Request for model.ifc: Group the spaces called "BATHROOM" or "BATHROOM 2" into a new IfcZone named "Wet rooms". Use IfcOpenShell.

First a look at what the model holds.

```python
import ifcopenshell

model = ifcopenshell.open("model.ifc")
print(model.schema)
seen = {}
for space in model.by_type("IfcSpace"):
    seen[space.LongName] = seen.get(space.LongName, 0) + 1
for name, count in sorted(seen.items(), key=str):
    print(count, "x", name)
print("zones:", [z.Name for z in model.by_type("IfcZone")][:20])
```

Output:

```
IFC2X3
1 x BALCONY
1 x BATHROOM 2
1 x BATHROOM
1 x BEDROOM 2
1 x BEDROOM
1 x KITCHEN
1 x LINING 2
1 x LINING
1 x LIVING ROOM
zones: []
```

```python
import ifcopenshell
import ifcopenshell.api.group
import ifcopenshell.api.root

model = ifcopenshell.open("model.ifc")

names = {"BATHROOM", "BATHROOM 2"}
spaces = [s for s in model.by_type("IfcSpace") if s.LongName in names]

zone = ifcopenshell.api.root.create_entity(model, ifc_class="IfcZone", name="Wet rooms")
ifcopenshell.api.group.assign_group(model, products=spaces, group=zone)
print(len(spaces), "spaces in", zone.Name)

model.write("model_v2.ifc")
```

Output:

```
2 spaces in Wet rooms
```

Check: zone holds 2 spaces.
